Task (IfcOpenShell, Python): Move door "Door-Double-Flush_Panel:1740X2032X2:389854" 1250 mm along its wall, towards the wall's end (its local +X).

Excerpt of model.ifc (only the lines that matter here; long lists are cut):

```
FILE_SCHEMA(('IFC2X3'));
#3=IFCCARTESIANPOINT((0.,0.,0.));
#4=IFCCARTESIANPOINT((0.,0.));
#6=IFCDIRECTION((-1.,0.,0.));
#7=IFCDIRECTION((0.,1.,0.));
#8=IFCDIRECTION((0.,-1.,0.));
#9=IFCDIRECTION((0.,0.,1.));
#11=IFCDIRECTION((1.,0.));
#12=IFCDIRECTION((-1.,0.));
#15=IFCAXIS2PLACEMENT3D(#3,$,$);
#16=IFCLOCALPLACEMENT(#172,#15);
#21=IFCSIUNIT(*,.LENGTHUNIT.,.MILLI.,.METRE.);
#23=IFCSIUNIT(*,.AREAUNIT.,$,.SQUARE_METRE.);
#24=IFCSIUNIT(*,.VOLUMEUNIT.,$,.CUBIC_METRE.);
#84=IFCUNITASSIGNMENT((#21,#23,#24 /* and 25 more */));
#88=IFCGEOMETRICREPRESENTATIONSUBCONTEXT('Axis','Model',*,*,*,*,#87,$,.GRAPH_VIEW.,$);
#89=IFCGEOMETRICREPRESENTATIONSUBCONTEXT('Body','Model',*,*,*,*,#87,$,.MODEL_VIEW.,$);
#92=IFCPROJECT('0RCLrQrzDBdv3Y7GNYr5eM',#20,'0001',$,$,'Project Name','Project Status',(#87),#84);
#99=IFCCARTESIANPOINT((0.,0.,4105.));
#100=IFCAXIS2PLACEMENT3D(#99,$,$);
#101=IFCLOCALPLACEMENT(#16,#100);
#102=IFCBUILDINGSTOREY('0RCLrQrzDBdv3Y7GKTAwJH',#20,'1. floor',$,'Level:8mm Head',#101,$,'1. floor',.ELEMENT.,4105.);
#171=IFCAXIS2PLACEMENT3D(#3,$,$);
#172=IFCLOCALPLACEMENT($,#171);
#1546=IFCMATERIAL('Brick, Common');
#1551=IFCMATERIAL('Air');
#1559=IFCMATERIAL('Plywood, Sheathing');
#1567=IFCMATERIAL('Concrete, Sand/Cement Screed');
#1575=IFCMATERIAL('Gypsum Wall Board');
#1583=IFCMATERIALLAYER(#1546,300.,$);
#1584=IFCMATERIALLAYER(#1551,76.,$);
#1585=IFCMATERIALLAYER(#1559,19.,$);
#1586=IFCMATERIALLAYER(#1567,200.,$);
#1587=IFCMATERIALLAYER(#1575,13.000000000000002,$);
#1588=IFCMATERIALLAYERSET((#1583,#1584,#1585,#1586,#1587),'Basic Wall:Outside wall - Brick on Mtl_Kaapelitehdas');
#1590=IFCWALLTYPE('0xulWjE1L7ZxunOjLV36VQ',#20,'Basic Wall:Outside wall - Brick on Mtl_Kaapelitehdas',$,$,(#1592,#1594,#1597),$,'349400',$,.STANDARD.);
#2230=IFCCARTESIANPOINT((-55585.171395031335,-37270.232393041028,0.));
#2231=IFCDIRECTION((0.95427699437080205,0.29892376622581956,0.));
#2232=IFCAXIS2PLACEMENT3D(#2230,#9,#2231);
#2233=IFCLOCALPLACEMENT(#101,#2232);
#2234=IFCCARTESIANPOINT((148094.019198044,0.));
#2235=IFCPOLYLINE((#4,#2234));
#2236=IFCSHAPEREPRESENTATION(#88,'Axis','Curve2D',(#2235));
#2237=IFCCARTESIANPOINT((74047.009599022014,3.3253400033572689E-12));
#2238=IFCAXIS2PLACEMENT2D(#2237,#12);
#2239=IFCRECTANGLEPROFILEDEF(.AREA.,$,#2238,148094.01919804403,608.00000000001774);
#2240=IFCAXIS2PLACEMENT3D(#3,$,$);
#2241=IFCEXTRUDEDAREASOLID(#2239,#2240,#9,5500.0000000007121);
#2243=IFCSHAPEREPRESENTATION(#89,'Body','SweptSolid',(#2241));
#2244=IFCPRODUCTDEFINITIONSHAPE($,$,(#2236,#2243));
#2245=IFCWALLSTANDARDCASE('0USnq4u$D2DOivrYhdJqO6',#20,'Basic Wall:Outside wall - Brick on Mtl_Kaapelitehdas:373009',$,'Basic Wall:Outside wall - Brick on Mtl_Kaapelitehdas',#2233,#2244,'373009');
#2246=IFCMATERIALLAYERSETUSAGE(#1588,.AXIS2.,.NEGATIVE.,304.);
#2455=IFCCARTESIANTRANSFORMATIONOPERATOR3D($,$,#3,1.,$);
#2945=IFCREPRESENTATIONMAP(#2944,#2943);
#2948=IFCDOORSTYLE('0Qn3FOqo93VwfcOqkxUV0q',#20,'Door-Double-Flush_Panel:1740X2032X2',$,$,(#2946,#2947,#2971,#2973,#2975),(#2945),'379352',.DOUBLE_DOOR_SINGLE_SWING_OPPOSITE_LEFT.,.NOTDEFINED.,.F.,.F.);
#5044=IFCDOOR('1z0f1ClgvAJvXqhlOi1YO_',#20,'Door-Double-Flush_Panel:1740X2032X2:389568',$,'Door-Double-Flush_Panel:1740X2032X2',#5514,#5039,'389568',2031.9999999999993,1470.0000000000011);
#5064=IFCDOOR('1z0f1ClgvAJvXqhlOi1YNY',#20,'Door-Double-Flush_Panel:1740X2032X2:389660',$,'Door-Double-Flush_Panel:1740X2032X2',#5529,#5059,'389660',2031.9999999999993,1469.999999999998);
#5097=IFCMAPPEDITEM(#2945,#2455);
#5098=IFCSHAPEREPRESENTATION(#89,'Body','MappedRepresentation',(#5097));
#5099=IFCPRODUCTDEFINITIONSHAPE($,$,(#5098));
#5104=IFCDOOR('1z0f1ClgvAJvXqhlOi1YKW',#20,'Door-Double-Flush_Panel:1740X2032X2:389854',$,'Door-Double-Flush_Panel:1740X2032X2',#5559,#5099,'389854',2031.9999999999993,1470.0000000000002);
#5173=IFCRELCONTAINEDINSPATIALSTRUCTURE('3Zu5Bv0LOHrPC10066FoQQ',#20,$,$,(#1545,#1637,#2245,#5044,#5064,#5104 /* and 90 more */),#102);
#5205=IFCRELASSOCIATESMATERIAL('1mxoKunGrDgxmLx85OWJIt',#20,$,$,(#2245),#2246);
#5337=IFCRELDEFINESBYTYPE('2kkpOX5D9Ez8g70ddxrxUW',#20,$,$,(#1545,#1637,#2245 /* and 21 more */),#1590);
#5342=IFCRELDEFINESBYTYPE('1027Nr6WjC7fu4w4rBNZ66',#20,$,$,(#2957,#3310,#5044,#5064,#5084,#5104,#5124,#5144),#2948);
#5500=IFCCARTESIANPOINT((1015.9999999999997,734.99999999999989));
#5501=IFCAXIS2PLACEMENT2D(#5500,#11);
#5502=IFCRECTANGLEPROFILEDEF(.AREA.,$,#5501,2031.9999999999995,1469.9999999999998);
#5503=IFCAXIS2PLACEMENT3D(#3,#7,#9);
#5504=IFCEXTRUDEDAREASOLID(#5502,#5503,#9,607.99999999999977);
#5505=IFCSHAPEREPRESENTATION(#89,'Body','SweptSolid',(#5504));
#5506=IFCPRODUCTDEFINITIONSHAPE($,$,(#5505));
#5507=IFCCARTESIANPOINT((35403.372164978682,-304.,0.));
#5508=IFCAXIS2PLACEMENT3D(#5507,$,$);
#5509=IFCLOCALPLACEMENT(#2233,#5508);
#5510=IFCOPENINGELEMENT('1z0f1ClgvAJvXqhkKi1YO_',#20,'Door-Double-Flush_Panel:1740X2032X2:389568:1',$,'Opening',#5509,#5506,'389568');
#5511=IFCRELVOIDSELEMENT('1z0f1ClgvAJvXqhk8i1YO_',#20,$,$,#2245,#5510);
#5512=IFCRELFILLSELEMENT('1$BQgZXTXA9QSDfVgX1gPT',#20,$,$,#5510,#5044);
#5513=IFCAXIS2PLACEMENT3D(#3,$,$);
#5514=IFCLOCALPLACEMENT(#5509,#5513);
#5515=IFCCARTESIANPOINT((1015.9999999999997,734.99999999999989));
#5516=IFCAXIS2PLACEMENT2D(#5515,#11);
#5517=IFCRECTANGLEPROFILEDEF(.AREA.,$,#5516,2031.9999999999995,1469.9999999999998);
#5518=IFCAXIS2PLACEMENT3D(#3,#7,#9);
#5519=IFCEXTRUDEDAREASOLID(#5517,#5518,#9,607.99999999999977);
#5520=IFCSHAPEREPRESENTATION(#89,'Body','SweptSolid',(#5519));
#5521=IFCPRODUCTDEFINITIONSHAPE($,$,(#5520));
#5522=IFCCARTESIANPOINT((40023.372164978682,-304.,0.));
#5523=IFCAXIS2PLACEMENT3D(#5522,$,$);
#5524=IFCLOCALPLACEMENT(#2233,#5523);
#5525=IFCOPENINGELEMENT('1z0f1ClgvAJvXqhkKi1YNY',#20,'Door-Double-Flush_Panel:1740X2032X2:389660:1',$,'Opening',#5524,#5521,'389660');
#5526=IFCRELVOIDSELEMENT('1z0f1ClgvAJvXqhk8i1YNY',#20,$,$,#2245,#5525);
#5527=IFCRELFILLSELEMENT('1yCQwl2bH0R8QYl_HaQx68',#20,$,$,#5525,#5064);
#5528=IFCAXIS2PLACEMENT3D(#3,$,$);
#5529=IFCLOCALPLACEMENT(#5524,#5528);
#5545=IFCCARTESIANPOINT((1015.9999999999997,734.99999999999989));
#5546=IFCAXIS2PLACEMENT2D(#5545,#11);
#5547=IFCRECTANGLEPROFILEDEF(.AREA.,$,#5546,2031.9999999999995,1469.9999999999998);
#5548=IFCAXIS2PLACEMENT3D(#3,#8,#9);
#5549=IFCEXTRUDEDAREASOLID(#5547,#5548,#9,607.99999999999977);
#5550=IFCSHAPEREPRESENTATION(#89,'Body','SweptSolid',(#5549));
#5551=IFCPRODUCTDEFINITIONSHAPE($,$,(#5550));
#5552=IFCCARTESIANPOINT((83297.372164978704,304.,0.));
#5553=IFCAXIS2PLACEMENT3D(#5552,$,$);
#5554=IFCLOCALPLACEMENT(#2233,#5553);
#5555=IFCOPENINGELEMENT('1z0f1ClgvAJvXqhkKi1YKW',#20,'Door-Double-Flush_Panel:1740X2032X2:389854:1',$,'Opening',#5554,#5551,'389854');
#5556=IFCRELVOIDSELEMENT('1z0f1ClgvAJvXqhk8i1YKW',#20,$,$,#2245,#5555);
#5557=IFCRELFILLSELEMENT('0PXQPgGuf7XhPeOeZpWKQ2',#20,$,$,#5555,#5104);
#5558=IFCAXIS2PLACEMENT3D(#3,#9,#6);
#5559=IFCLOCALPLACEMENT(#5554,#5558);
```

```python
import ifcopenshell
import ifcopenshell.api.geometry
import ifcopenshell.util.placement
import ifcopenshell.util.unit

model = ifcopenshell.open("model.ifc")
unit_scale = ifcopenshell.util.unit.calculate_unit_scale(model)

door = model.by_guid("1z0f1ClgvAJvXqhlOi1YKW")
opening = door.FillsVoids[0].RelatingOpeningElement
wall = opening.VoidsElements[0].RelatingBuildingElement

wall_matrix = ifcopenshell.util.placement.get_local_placement(wall.ObjectPlacement)
shift = wall_matrix[:3, 0] * 1.25 / unit_scale
before = ifcopenshell.util.placement.get_local_placement(door.ObjectPlacement)[:3, 3].copy()

# The door is placed relative to its opening, so it follows when the opening moves.
matrix = ifcopenshell.util.placement.get_local_placement(opening.ObjectPlacement)
matrix[:3, 3] += shift
ifcopenshell.api.geometry.edit_object_placement(
    model, product=opening, matrix=matrix, is_si=False, should_transform_children=True
)

after = ifcopenshell.util.placement.get_local_placement(door.ObjectPlacement)[:3, 3]
print("door moved by", (after - before).round(3) + 0.0)

model.write("model-out.ifc")
```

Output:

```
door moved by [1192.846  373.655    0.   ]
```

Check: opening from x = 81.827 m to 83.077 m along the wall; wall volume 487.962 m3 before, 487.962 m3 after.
